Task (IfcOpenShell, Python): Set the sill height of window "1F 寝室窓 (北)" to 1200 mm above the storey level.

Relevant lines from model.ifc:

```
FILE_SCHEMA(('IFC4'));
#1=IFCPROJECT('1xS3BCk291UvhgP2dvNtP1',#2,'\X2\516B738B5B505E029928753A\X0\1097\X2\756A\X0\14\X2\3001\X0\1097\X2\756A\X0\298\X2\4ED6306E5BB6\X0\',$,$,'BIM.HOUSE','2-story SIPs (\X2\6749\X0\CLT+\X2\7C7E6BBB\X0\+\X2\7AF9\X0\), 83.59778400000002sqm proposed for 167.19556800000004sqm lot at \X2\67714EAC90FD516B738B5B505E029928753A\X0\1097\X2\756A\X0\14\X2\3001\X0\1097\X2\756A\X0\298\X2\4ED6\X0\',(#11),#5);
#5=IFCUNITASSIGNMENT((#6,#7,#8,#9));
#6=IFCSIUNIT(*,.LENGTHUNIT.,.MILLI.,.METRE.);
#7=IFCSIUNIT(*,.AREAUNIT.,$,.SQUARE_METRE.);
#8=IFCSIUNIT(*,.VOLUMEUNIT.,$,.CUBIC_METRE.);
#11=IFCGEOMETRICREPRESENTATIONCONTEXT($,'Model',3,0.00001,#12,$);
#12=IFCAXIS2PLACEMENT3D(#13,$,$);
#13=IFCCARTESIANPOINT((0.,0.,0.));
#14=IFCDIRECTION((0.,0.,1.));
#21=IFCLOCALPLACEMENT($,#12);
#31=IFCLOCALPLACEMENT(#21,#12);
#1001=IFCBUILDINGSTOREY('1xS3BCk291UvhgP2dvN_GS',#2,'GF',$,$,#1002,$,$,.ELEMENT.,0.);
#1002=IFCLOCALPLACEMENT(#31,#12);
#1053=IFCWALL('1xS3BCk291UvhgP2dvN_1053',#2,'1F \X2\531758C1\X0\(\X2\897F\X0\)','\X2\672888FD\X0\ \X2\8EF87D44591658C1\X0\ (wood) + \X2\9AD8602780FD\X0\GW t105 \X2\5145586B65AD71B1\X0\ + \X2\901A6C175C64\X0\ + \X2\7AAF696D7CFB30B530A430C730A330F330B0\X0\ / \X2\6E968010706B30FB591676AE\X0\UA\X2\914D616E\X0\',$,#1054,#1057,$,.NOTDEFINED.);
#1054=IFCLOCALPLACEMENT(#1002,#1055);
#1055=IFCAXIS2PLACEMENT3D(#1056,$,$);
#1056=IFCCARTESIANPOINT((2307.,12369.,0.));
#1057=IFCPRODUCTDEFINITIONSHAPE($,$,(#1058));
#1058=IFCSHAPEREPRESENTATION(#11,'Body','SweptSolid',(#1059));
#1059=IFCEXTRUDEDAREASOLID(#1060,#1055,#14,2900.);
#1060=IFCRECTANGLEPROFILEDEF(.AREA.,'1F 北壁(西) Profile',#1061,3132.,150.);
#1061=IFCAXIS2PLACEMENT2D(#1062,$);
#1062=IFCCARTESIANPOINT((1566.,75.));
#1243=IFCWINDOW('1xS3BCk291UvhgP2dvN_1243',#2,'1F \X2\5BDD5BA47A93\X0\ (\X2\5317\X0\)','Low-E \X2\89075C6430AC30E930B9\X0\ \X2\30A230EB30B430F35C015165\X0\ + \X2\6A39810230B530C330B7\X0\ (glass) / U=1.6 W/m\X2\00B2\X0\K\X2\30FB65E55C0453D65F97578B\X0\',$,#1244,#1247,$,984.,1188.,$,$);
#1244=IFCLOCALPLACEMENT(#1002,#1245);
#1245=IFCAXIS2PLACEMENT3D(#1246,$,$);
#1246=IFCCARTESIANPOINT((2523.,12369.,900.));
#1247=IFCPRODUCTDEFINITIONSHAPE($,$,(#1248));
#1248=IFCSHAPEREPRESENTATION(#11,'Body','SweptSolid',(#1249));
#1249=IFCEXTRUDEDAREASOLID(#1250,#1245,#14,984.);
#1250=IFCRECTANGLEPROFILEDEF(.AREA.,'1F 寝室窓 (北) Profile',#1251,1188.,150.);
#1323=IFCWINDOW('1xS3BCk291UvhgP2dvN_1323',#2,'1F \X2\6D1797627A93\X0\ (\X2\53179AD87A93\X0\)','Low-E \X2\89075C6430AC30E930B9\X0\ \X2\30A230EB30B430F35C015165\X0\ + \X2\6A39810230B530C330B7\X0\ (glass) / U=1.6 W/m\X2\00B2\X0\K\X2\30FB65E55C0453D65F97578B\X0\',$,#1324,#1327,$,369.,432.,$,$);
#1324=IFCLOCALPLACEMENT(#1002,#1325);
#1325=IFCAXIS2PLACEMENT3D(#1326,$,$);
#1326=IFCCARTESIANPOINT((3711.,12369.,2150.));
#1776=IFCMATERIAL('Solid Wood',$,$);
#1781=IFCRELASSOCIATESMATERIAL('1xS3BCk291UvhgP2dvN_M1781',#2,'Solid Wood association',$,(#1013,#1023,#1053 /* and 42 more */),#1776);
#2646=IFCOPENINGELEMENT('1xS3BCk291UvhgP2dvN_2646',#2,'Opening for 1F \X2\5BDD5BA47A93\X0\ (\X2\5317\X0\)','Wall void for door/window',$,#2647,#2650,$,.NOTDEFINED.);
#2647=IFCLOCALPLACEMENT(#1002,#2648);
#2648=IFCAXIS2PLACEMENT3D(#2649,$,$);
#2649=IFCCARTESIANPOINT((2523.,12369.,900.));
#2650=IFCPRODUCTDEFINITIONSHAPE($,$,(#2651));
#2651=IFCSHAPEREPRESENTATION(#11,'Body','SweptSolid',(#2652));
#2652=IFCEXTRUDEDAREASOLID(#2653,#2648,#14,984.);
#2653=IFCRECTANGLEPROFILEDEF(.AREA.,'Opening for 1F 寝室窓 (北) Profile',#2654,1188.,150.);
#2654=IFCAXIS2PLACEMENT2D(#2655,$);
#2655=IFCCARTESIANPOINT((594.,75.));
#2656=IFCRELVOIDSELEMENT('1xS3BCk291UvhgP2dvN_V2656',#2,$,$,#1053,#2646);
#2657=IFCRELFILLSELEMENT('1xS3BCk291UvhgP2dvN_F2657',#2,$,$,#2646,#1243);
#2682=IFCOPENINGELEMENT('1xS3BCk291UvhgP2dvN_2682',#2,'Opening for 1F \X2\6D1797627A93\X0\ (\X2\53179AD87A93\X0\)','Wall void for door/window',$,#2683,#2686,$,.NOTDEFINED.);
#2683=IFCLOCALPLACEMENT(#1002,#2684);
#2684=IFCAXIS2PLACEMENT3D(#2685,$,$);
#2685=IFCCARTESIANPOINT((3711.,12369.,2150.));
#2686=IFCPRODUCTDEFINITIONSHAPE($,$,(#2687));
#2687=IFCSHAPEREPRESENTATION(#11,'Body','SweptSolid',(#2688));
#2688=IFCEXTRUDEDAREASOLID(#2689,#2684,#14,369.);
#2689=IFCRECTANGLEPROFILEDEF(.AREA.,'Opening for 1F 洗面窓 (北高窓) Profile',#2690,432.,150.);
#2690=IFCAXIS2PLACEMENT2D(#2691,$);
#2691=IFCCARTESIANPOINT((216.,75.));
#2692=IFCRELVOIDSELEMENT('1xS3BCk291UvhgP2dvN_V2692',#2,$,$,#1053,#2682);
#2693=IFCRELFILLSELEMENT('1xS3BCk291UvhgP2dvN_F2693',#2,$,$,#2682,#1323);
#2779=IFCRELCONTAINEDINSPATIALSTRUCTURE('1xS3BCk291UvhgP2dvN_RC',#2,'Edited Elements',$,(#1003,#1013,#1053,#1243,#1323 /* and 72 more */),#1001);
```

```python
import numpy as np
import ifcopenshell
import ifcopenshell.api.geometry
import ifcopenshell.geom
import ifcopenshell.util.element
import ifcopenshell.util.placement
import ifcopenshell.util.shape
import ifcopenshell.util.unit

model = ifcopenshell.open("model.ifc")
unit_scale = ifcopenshell.util.unit.calculate_unit_scale(model)

window = model.by_guid("1xS3BCk291UvhgP2dvN_1243")
opening = window.FillsVoids[0].RelatingOpeningElement
storey = ifcopenshell.util.element.get_container(window, ifc_class="IfcBuildingStorey")
level = ifcopenshell.util.placement.get_local_placement(storey.ObjectPlacement)[2, 3]

# The opening's origin need not be at the sill, so measure its lowest point.
shape = ifcopenshell.geom.create_shape(ifcopenshell.geom.settings(), opening)
bottom = ifcopenshell.util.shape.get_shape_bottom_elevation(shape, shape.geometry) / unit_scale
dz = level + 1.2 / unit_scale - bottom

shift = np.array([0.0, 0.0, dz])
# The window is not placed relative to its opening, so move both.
for product in (opening, window):
    matrix = ifcopenshell.util.placement.get_local_placement(product.ObjectPlacement)
    matrix[:3, 3] += shift
    ifcopenshell.api.geometry.edit_object_placement(model, product=product, matrix=matrix, is_si=False)

print(f"moved by {dz * unit_scale:+.3f} m")

model.write("model_rev.ifc")
```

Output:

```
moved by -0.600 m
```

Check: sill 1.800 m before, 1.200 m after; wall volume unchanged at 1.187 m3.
